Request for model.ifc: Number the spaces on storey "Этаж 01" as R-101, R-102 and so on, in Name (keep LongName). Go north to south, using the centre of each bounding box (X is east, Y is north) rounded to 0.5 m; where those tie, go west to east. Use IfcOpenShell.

First a look at what the model holds.

```python
import ifcopenshell
import ifcopenshell.util.element
import ifcopenshell.util.placement

model = ifcopenshell.open("model.ifc")
print(model.schema)
storey = next(s for s in model.by_type("IfcBuildingStorey") if s.Name == "Этаж 01")
spaces = [e for e in ifcopenshell.util.element.get_decomposition(storey) if e.is_a("IfcSpace")]
for e in sorted(spaces, key=lambda e: e.id()):
    origin = ifcopenshell.util.placement.get_local_placement(e.ObjectPlacement)[:3, 3]
    print(e.id(), e.Name, e.LongName, origin.round(2) + 0.0, sep=" | ")
```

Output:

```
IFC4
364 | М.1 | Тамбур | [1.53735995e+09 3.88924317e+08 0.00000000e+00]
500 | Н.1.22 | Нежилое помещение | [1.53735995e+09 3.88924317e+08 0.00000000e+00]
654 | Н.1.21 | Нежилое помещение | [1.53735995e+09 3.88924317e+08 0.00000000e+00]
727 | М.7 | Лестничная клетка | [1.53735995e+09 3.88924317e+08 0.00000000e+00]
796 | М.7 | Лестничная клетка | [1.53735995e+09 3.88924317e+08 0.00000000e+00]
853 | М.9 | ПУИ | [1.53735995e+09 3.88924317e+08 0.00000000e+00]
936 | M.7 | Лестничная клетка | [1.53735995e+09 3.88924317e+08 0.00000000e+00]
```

```python
import ifcopenshell
import ifcopenshell.geom
import ifcopenshell.util.element
import ifcopenshell.util.shape

model = ifcopenshell.open("model.ifc")
settings = ifcopenshell.geom.settings()
settings.set("use-world-coords", True)


def centre(element):
    shape = ifcopenshell.geom.create_shape(settings, element)
    return ifcopenshell.util.shape.get_bbox_centroid(shape.geometry)


storey = next(s for s in model.by_type("IfcBuildingStorey") if s.Name == "Этаж 01")
spaces = [e for e in ifcopenshell.util.element.get_decomposition(storey) if e.is_a("IfcSpace")]

# Insertion points can sit at a corner or the storey origin, so sort by the geometry (in metres).
centres = {e: centre(e) for e in spaces}
spaces.sort(key=lambda e: (-round(centres[e][1] / 0.5), centres[e][0]))

for i, e in enumerate(spaces, start=1):
    number = f"R-1{i:02d}"
    e.Name = number
    print(e.id(), number)

model.write("model_v2.ifc")
```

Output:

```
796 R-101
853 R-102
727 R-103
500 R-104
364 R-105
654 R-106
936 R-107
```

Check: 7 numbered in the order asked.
